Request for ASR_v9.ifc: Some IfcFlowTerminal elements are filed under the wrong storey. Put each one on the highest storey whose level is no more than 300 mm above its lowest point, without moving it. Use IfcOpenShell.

First a look at what the model holds.

```python
import ifcopenshell
import ifcopenshell.util.element
import ifcopenshell.util.placement

model = ifcopenshell.open("ASR_v9.ifc")
print(model.schema)
for storey in model.by_type("IfcBuildingStorey"):
    level = ifcopenshell.util.placement.get_storey_elevation(storey)
    count = sum(e.is_a("IfcFlowTerminal") for e in ifcopenshell.util.element.get_contained(storey))
    print(storey.id(), storey.Name, round(level, 3), count, sep=" | ")
```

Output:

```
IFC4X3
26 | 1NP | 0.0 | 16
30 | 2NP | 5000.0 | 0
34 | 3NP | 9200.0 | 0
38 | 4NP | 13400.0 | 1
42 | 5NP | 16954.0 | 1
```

```python
import ifcopenshell
import ifcopenshell.api.spatial
import ifcopenshell.geom
import ifcopenshell.util.element
import ifcopenshell.util.placement
import ifcopenshell.util.shape
import ifcopenshell.util.unit

model = ifcopenshell.open("ASR_v9.ifc")
unit_scale = ifcopenshell.util.unit.calculate_unit_scale(model)
settings = ifcopenshell.geom.settings()

levels = sorted(
    ((ifcopenshell.util.placement.get_storey_elevation(s) * unit_scale, s) for s in model.by_type("IfcBuildingStorey")),
    key=lambda pair: pair[0],
)

for e in model.by_type("IfcFlowTerminal"):
    current = e.ContainedInStructure[0].RelatingStructure if e.ContainedInStructure else None
    if current is None or not current.is_a("IfcBuildingStorey"):
        continue
    shape = ifcopenshell.geom.create_shape(settings, e)
    bottom = ifcopenshell.util.shape.get_shape_bottom_elevation(shape, shape.geometry)
    below = [s for level, s in levels if level <= bottom + 0.3]
    storey = below[-1] if below else levels[0][1]
    if storey != current:
        # assign_container keeps the world position.
        ifcopenshell.api.spatial.assign_container(model, products=[e], relating_structure=storey)
        print(e.id(), current.Name, "->", storey.Name)

model.write("ASR_v9_updated.ifc")
```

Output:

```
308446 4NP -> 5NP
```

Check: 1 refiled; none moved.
